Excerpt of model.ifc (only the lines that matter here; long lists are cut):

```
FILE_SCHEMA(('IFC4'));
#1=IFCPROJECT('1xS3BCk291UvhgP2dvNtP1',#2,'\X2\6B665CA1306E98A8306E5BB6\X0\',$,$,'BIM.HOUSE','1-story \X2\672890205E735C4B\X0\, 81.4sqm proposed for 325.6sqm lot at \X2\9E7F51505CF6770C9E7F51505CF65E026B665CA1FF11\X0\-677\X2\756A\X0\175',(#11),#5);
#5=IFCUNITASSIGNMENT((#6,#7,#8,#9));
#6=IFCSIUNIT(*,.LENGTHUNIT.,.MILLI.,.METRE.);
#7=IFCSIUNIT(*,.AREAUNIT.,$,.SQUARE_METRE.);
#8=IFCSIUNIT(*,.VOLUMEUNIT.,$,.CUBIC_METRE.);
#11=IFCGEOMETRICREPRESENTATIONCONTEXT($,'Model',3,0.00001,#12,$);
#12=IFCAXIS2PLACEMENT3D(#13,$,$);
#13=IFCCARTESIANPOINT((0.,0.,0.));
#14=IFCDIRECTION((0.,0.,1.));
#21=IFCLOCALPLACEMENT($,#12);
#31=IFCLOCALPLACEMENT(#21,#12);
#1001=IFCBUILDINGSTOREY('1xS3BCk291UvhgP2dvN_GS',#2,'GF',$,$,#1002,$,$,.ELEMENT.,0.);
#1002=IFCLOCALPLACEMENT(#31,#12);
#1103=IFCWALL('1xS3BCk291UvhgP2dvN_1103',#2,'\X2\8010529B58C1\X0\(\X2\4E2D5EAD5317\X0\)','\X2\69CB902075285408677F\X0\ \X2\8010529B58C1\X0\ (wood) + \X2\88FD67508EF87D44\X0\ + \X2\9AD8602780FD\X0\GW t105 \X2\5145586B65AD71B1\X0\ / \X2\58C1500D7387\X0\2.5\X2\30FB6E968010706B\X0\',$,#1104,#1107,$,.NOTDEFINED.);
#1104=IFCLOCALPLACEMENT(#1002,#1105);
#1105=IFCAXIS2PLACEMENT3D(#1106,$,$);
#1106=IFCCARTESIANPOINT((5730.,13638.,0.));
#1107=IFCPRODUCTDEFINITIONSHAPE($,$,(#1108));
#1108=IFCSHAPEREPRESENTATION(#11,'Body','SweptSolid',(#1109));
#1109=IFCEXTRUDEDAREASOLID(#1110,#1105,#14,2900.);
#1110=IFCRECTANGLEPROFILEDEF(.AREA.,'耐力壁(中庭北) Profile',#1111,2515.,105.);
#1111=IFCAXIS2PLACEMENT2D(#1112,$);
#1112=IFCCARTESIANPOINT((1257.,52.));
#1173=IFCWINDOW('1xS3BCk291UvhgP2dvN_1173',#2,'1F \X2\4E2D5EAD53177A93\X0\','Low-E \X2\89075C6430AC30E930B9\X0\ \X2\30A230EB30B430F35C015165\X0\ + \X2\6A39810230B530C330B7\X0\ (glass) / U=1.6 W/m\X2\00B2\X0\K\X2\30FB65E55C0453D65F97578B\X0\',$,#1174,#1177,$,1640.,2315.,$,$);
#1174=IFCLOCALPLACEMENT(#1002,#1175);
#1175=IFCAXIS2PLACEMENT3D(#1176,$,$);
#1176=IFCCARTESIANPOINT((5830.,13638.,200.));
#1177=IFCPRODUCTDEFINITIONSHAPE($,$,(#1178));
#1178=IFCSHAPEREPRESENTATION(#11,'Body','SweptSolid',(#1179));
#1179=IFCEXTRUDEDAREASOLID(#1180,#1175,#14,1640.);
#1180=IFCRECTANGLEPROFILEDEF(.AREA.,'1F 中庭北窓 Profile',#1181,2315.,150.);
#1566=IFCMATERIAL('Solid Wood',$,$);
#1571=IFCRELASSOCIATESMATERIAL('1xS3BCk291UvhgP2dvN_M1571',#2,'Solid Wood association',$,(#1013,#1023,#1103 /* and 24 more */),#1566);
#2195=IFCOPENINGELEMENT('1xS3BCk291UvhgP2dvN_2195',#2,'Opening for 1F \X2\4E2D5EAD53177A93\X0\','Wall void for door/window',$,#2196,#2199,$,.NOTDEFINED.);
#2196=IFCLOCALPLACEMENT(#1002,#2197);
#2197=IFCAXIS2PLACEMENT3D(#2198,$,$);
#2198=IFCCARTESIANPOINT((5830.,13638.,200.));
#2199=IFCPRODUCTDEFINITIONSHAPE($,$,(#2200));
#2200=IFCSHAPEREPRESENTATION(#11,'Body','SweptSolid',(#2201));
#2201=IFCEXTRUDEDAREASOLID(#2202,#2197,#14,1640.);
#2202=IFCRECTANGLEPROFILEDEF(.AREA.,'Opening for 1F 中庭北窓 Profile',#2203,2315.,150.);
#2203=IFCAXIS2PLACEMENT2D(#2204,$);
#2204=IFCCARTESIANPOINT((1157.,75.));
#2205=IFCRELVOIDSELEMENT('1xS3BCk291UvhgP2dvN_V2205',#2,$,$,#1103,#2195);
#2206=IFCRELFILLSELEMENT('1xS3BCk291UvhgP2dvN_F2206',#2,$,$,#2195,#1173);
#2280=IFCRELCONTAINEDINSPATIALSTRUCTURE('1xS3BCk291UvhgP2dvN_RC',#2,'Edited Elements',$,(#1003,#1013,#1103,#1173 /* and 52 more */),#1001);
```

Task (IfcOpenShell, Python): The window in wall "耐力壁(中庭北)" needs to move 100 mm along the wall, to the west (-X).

```python
import ifcopenshell
import ifcopenshell.api.geometry
import ifcopenshell.util.placement
import ifcopenshell.util.unit

model = ifcopenshell.open("model.ifc")
unit_scale = ifcopenshell.util.unit.calculate_unit_scale(model)

window = model.by_guid("1xS3BCk291UvhgP2dvN_1173")
opening = window.FillsVoids[0].RelatingOpeningElement
wall = opening.VoidsElements[0].RelatingBuildingElement

wall_matrix = ifcopenshell.util.placement.get_local_placement(wall.ObjectPlacement)
shift = wall_matrix[:3, 0] * -0.1 / unit_scale
before = ifcopenshell.util.placement.get_local_placement(window.ObjectPlacement)[:3, 3].copy()

# The window is not placed relative to its opening, so move both.
for product in (opening, window):
    matrix = ifcopenshell.util.placement.get_local_placement(product.ObjectPlacement)
    matrix[:3, 3] += shift
    ifcopenshell.api.geometry.edit_object_placement(model, product=product, matrix=matrix, is_si=False)

after = ifcopenshell.util.placement.get_local_placement(window.ObjectPlacement)[:3, 3]
print("window moved by", (after - before).round(3) + 0.0)

model.write("model_edited.ifc")
```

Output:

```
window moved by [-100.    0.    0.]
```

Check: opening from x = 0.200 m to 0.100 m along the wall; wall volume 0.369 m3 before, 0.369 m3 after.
